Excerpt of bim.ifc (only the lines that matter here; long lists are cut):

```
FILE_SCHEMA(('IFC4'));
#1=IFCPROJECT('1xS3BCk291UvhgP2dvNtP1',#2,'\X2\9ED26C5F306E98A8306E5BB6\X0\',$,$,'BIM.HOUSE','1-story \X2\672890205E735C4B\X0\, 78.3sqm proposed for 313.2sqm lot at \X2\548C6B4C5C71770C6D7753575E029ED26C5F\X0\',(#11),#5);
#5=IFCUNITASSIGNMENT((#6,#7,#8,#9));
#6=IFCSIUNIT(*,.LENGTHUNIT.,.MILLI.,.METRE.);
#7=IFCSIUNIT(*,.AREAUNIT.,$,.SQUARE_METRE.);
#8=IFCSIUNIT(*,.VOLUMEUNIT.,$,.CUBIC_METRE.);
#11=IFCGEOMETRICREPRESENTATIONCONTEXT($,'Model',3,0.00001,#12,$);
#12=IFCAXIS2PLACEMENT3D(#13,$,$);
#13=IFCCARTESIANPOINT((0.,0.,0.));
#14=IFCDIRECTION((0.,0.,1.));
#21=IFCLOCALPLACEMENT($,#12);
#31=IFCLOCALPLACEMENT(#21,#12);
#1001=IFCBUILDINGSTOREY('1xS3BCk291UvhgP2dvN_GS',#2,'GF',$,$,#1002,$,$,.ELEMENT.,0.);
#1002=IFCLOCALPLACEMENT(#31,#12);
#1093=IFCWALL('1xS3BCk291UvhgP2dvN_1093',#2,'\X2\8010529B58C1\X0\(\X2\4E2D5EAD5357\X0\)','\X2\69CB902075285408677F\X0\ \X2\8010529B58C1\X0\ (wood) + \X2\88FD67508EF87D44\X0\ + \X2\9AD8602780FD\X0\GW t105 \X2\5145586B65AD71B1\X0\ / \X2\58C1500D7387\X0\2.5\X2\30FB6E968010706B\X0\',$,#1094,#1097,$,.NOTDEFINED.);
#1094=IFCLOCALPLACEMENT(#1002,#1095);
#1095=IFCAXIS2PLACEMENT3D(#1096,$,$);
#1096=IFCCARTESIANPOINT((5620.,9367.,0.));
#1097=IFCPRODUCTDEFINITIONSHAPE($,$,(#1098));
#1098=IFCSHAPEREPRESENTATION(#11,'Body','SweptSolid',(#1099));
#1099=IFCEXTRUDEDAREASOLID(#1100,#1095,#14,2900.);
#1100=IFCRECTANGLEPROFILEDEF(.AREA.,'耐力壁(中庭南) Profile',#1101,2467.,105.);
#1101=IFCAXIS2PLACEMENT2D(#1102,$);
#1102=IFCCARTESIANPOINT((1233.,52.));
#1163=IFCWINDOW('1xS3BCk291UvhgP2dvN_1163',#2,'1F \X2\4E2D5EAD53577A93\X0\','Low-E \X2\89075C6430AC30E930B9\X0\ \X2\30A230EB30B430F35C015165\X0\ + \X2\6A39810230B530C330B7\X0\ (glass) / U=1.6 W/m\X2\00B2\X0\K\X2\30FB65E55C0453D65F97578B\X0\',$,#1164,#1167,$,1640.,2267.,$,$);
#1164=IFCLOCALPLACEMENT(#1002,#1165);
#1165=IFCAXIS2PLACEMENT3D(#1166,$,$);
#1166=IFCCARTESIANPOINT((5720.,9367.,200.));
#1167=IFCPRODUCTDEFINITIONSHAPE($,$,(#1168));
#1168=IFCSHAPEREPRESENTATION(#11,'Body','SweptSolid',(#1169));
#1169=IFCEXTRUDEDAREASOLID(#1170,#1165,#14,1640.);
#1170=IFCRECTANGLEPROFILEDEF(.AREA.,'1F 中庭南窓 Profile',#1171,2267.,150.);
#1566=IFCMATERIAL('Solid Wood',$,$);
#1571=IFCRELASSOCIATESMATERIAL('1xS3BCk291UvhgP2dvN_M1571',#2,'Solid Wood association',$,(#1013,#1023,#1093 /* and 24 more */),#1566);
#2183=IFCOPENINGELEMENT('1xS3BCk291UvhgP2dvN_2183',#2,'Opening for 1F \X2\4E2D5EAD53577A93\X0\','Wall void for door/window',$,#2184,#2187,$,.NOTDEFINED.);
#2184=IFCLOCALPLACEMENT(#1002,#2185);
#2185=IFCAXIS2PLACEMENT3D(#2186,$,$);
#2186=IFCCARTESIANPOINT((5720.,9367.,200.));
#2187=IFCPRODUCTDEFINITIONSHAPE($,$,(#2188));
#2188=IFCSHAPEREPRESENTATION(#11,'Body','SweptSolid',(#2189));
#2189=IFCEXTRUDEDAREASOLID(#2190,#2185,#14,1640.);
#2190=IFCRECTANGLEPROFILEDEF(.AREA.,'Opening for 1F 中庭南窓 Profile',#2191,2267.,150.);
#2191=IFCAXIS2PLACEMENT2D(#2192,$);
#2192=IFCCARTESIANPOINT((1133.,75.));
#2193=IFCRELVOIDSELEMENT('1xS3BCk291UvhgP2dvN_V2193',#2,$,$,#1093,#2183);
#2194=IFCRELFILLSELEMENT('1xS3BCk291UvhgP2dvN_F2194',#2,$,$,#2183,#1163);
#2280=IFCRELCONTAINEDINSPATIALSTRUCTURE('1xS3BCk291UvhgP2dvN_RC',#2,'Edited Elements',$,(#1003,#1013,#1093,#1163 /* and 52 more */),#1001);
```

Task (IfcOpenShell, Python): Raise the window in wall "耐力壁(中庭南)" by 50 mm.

```python
import numpy as np
import ifcopenshell
import ifcopenshell.api.geometry
import ifcopenshell.util.placement
import ifcopenshell.util.unit

model = ifcopenshell.open("bim.ifc")
unit_scale = ifcopenshell.util.unit.calculate_unit_scale(model)

window = model.by_id(1163)
opening = window.FillsVoids[0].RelatingOpeningElement
dz = 0.05 / unit_scale

shift = np.array([0.0, 0.0, dz])
# The window is not placed relative to its opening, so move both.
for product in (opening, window):
    matrix = ifcopenshell.util.placement.get_local_placement(product.ObjectPlacement)
    matrix[:3, 3] += shift
    ifcopenshell.api.geometry.edit_object_placement(model, product=product, matrix=matrix, is_si=False)

print(f"moved by {dz * unit_scale:+.3f} m")

model.write("bim_updated.ifc")
```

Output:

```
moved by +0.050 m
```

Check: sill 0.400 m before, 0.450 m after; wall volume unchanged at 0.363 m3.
